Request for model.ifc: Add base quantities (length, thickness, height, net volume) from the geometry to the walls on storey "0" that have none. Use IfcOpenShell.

First a look at what the model holds.

```python
import ifcopenshell
import ifcopenshell.util.element
import ifcopenshell.util.unit

model = ifcopenshell.open("model.ifc")
print(model.schema)
for unit_type in ("LENGTHUNIT", "AREAUNIT", "VOLUMEUNIT"):
    print(unit_type, ifcopenshell.util.unit.calculate_unit_scale(model, unit_type))
storey = next(s for s in model.by_type("IfcBuildingStorey") if s.Name == "0")
walls = [e for e in ifcopenshell.util.element.get_decomposition(storey) if e.is_a("IfcWall")]
for e in sorted(walls, key=lambda e: e.id()):
    print(e.id(), e.is_a(), e.Name, list(ifcopenshell.util.element.get_psets(e, qtos_only=True)), sep=" | ")
```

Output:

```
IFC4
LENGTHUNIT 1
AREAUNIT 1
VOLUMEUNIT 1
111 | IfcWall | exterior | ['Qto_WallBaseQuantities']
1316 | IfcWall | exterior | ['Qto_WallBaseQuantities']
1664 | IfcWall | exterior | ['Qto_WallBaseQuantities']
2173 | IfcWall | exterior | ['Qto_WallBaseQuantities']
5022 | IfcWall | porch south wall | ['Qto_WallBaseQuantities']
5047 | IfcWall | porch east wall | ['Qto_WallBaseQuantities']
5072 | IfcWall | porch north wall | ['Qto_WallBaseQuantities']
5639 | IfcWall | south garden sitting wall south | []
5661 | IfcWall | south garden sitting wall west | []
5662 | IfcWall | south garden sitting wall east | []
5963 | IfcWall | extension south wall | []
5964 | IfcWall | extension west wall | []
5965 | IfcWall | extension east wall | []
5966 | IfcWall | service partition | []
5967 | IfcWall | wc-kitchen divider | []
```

```python
import ifcopenshell
import ifcopenshell.api.pset
import ifcopenshell.geom
import ifcopenshell.util.element
import ifcopenshell.util.shape
import ifcopenshell.util.unit

model = ifcopenshell.open("model.ifc")
unit_scale = ifcopenshell.util.unit.calculate_unit_scale(model)
volume_scale = ifcopenshell.util.unit.calculate_unit_scale(model, "VOLUMEUNIT")
settings = ifcopenshell.geom.settings()

storey = next(s for s in model.by_type("IfcBuildingStorey") if s.Name == "0")
walls = [e for e in ifcopenshell.util.element.get_decomposition(storey) if e.is_a("IfcWall")]

for e in sorted(walls, key=lambda e: e.id()):
    if ifcopenshell.util.element.get_psets(e, qtos_only=True, should_inherit=False):
        continue
    # Geometry comes back in metres, in the element's own axes.
    shape = ifcopenshell.geom.create_shape(settings, e)
    values = {
        "Length": ifcopenshell.util.shape.get_x(shape.geometry) / unit_scale,
        "Width": ifcopenshell.util.shape.get_y(shape.geometry) / unit_scale,
        "Height": ifcopenshell.util.shape.get_z(shape.geometry) / unit_scale,
        "NetVolume": ifcopenshell.util.shape.get_volume(shape.geometry) / volume_scale,
    }
    qto = ifcopenshell.api.pset.add_qto(model, product=e, name="Qto_WallBaseQuantities")
    ifcopenshell.api.pset.edit_qto(model, qto=qto, properties=values)
    print(e.id(), {k: round(v, 3) for k, v in values.items()})

model.write("model_v2.ifc")
```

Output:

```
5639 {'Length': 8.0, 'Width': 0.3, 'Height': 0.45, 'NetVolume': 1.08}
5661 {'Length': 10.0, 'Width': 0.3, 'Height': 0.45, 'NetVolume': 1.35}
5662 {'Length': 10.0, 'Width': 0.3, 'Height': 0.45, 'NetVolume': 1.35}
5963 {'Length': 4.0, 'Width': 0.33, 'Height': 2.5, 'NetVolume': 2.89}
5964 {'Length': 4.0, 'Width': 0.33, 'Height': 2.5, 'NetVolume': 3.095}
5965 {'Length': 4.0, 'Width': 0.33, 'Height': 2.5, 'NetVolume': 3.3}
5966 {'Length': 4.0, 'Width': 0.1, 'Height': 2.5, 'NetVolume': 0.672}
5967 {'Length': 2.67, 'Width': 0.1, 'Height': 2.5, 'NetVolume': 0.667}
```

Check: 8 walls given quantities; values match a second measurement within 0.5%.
